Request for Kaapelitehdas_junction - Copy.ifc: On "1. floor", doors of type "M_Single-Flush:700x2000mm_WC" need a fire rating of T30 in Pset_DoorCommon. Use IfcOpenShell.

First a look at what the model holds.

```python
import ifcopenshell
import ifcopenshell.util.element

model = ifcopenshell.open("Kaapelitehdas_junction - Copy.ifc")
print(model.schema)
storey = next(s for s in model.by_type("IfcBuildingStorey") if s.Name == "1. floor")
doors = [e for e in ifcopenshell.util.element.get_decomposition(storey) if e.is_a("IfcDoor")]
seen = {}
for e in doors:
    element_type = ifcopenshell.util.element.get_type(e)
    key = (element_type.Name if element_type != e and element_type else None, ifcopenshell.util.element.get_pset(e, "Pset_DoorCommon", "FireRating"))
    seen[key] = seen.get(key, 0) + 1
for (name, value), count in sorted(seen.items(), key=str):
    print(count, "x", name, "|", value)
```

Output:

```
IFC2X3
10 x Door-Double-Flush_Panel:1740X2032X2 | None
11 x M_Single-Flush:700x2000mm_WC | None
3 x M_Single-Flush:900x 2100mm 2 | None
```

```python
import ifcopenshell
import ifcopenshell.api.pset
import ifcopenshell.util.element

model = ifcopenshell.open("Kaapelitehdas_junction - Copy.ifc")

storey = next(s for s in model.by_type("IfcBuildingStorey") if s.Name == "1. floor")
doors = [e for e in ifcopenshell.util.element.get_decomposition(storey) if e.is_a("IfcDoor")]

count = 0
for e in doors:
    element_type = ifcopenshell.util.element.get_type(e)
    if element_type in (None, e) or element_type.Name != "M_Single-Flush:700x2000mm_WC":
        continue
    # add_pset returns the element's existing set when there is one.
    pset = ifcopenshell.api.pset.add_pset(model, product=e, name="Pset_DoorCommon")
    ifcopenshell.api.pset.edit_pset(model, pset=pset, properties={"FireRating": "T30"})
    count += 1

print(count, "doors updated")

model.write("Kaapelitehdas_junction - Copy_updated.ifc")
```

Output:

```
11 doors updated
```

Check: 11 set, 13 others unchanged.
